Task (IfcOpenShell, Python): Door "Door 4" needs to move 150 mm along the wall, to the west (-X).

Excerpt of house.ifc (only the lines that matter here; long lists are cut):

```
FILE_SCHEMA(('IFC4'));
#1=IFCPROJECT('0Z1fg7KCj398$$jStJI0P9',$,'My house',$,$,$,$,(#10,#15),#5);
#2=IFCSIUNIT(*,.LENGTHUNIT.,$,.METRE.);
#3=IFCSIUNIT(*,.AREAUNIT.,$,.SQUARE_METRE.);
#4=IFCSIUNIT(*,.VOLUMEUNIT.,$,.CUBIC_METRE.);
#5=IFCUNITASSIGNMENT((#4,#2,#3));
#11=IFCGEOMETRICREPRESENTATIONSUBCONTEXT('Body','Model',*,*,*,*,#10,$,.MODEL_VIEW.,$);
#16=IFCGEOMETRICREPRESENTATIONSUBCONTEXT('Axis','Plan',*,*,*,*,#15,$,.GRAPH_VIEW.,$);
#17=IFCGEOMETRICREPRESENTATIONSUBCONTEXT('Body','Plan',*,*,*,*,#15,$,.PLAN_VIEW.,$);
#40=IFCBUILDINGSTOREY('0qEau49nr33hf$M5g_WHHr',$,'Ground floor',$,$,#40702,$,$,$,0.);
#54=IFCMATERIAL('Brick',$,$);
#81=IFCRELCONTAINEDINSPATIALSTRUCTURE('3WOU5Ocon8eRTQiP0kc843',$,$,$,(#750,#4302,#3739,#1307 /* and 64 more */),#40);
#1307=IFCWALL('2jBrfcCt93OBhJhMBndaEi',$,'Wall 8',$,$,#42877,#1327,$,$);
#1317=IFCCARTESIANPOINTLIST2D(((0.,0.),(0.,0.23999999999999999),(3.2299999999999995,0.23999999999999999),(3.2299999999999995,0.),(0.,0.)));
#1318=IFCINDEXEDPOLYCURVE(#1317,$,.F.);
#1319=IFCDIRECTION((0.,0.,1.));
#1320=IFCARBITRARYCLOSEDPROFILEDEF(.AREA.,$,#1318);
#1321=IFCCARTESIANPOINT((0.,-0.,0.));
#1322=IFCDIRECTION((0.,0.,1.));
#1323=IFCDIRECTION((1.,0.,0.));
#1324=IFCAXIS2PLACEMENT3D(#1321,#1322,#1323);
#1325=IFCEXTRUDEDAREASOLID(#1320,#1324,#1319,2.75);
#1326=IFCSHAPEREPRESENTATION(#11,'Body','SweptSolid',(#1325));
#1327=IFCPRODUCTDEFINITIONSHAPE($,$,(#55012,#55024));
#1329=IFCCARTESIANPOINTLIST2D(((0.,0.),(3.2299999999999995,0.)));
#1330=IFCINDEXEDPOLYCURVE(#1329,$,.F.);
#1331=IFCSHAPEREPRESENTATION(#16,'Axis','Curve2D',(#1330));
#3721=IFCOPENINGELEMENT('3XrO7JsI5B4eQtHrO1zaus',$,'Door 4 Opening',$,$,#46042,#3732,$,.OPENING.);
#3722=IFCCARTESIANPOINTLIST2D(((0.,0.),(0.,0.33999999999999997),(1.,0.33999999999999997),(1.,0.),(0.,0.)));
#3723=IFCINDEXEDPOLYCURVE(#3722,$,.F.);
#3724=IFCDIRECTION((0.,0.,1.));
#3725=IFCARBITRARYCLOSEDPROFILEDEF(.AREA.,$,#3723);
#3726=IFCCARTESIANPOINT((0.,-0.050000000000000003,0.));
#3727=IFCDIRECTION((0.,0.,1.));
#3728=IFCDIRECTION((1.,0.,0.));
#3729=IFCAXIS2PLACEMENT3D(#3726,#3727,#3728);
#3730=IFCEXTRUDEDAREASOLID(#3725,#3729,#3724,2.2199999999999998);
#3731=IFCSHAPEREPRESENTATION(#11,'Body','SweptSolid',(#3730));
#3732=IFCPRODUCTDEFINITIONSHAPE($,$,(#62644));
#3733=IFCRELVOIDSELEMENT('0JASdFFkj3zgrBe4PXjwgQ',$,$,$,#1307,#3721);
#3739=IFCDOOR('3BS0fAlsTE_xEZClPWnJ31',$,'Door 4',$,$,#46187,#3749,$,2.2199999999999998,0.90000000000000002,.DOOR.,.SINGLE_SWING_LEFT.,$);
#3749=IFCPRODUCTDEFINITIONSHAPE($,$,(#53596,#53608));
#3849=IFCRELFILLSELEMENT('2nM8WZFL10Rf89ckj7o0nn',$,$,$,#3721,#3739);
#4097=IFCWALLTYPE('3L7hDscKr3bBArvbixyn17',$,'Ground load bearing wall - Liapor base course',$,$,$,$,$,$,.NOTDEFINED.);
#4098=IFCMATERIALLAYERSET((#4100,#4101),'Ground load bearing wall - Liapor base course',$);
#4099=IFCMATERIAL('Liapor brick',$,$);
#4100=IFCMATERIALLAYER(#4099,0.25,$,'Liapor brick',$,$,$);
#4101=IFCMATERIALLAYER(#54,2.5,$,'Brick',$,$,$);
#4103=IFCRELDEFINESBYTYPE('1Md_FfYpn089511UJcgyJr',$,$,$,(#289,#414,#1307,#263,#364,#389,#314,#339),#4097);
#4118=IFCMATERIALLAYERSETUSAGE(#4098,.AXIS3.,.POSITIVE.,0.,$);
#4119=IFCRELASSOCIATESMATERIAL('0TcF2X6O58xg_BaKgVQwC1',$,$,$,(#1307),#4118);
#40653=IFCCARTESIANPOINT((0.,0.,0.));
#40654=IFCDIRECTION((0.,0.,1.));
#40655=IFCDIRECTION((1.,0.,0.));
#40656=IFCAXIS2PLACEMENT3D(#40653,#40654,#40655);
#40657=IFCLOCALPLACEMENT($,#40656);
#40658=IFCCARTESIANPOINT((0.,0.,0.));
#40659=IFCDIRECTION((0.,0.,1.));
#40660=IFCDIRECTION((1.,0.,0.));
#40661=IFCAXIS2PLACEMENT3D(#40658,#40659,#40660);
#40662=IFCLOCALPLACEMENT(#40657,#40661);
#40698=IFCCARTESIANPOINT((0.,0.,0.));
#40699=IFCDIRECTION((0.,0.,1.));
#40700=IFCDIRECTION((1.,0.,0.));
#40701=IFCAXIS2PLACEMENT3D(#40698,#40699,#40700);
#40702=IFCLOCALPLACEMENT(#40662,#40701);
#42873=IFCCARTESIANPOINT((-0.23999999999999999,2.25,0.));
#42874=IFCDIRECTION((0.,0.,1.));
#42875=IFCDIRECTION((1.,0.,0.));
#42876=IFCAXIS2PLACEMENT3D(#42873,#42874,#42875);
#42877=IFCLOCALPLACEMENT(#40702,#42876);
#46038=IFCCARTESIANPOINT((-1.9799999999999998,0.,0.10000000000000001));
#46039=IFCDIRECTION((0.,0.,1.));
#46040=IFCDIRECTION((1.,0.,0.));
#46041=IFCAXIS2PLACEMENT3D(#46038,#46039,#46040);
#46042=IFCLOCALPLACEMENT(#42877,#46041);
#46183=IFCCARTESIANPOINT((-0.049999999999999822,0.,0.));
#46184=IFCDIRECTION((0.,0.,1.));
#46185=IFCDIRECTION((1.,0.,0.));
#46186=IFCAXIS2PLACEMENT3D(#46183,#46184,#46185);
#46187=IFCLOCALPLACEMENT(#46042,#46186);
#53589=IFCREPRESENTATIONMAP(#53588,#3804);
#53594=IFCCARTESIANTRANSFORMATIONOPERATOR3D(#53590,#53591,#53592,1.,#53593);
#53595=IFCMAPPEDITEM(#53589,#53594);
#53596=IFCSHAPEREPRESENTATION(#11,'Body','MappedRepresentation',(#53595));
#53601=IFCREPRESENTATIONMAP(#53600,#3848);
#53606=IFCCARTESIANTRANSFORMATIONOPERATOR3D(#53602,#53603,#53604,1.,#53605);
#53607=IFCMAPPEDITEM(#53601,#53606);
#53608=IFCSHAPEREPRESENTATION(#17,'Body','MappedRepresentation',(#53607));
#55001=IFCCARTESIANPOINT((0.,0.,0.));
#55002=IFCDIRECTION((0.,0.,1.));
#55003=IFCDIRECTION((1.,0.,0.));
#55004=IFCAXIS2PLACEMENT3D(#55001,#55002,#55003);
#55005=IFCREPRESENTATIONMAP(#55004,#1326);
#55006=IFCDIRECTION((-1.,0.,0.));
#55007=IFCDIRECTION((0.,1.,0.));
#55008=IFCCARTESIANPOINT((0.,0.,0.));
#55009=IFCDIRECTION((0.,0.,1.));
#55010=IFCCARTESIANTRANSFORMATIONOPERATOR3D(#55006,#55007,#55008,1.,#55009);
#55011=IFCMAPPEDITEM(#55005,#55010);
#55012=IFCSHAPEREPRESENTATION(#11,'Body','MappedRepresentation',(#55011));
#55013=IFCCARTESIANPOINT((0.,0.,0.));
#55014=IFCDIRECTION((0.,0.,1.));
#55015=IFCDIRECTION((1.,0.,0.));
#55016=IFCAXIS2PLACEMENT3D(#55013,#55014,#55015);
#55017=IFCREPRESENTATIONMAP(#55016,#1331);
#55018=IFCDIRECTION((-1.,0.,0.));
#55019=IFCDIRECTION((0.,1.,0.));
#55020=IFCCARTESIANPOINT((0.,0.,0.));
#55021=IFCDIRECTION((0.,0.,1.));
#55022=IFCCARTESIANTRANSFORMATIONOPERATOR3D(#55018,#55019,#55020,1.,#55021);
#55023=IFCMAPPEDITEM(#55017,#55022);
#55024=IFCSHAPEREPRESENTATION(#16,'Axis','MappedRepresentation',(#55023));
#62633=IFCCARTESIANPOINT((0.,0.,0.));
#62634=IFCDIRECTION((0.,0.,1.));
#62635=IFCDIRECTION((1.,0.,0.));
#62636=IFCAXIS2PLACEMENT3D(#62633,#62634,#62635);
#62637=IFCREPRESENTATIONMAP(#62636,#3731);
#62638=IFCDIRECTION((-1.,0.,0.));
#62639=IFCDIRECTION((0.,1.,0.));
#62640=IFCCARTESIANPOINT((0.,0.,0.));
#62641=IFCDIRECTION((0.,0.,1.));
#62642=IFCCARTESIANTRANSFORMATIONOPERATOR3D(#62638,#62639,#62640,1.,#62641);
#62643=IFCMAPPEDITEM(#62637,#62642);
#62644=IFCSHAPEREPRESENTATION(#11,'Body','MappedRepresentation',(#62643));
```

```python
import ifcopenshell
import ifcopenshell.api.geometry
import ifcopenshell.util.placement
import ifcopenshell.util.unit

model = ifcopenshell.open("house.ifc")
unit_scale = ifcopenshell.util.unit.calculate_unit_scale(model)

door = model.by_guid("3BS0fAlsTE_xEZClPWnJ31")
opening = door.FillsVoids[0].RelatingOpeningElement
wall = opening.VoidsElements[0].RelatingBuildingElement

wall_matrix = ifcopenshell.util.placement.get_local_placement(wall.ObjectPlacement)
shift = wall_matrix[:3, 0] * -0.15 / unit_scale
before = ifcopenshell.util.placement.get_local_placement(door.ObjectPlacement)[:3, 3].copy()

# The door is placed relative to its opening, so it follows when the opening moves.
matrix = ifcopenshell.util.placement.get_local_placement(opening.ObjectPlacement)
matrix[:3, 3] += shift
ifcopenshell.api.geometry.edit_object_placement(
    model, product=opening, matrix=matrix, is_si=False, should_transform_children=True
)

after = ifcopenshell.util.placement.get_local_placement(door.ObjectPlacement)[:3, 3]
print("door moved by", (after - before).round(3) + 0.0)

model.write("house_v2.ifc")
```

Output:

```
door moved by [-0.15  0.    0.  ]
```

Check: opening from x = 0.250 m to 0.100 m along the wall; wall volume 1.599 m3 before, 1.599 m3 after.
